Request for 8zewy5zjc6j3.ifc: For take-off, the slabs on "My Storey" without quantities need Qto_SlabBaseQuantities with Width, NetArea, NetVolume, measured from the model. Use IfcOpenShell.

First a look at what the model holds.

```python
import ifcopenshell
import ifcopenshell.util.element
import ifcopenshell.util.unit

model = ifcopenshell.open("8zewy5zjc6j3.ifc")
print(model.schema)
for unit_type in ("LENGTHUNIT", "AREAUNIT", "VOLUMEUNIT"):
    print(unit_type, ifcopenshell.util.unit.calculate_unit_scale(model, unit_type))
storey = next(s for s in model.by_type("IfcBuildingStorey") if s.Name == "My Storey")
slabs = [e for e in ifcopenshell.util.element.get_decomposition(storey) if e.is_a("IfcSlab")]
for e in sorted(slabs, key=lambda e: e.id()):
    print(e.id(), e.is_a(), e.Name, list(ifcopenshell.util.element.get_psets(e, qtos_only=True)), sep=" | ")
```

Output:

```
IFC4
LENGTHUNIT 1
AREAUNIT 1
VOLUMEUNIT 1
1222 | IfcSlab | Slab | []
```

```python
import ifcopenshell
import ifcopenshell.api.pset
import ifcopenshell.geom
import ifcopenshell.util.element
import ifcopenshell.util.shape
import ifcopenshell.util.unit

model = ifcopenshell.open("8zewy5zjc6j3.ifc")
unit_scale = ifcopenshell.util.unit.calculate_unit_scale(model)
area_scale = ifcopenshell.util.unit.calculate_unit_scale(model, "AREAUNIT")
volume_scale = ifcopenshell.util.unit.calculate_unit_scale(model, "VOLUMEUNIT")
settings = ifcopenshell.geom.settings()

storey = next(s for s in model.by_type("IfcBuildingStorey") if s.Name == "My Storey")
slabs = [e for e in ifcopenshell.util.element.get_decomposition(storey) if e.is_a("IfcSlab")]

for e in sorted(slabs, key=lambda e: e.id()):
    if ifcopenshell.util.element.get_psets(e, qtos_only=True, should_inherit=False):
        continue
    # Geometry comes back in metres, in the element's own axes.
    shape = ifcopenshell.geom.create_shape(settings, e)
    values = {
        "Width": ifcopenshell.util.shape.get_z(shape.geometry) / unit_scale,
        "NetArea": ifcopenshell.util.shape.get_footprint_area(shape.geometry) / area_scale,
        "NetVolume": ifcopenshell.util.shape.get_volume(shape.geometry) / volume_scale,
    }
    qto = ifcopenshell.api.pset.add_qto(model, product=e, name="Qto_SlabBaseQuantities")
    ifcopenshell.api.pset.edit_qto(model, qto=qto, properties=values)
    print(e.id(), {k: round(v, 3) for k, v in values.items()})

model.write("8zewy5zjc6j3_rev.ifc")
```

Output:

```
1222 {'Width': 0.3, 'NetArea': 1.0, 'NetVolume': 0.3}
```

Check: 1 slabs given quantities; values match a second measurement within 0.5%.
